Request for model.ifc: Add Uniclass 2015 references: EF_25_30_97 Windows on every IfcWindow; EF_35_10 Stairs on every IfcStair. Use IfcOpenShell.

First a look at what the model holds.

```python
import ifcopenshell

model = ifcopenshell.open("model.ifc")
print(model.schema)
print("classifications:", [c.Name for c in model.by_type("IfcClassification")])
for ifc_class in ("IfcDoor", "IfcRoof", "IfcStair", "IfcWall", "IfcWindow"):
    print(ifc_class, len(model.by_type(ifc_class)))
```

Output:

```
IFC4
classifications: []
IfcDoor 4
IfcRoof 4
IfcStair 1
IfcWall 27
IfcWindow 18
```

```python
import ifcopenshell
import ifcopenshell.api.classification

model = ifcopenshell.open("model.ifc")

system = ifcopenshell.api.classification.add_classification(model, classification="Uniclass 2015")

codes = {
    "IfcWindow": ("EF_25_30_97", "Windows"),
    "IfcStair": ("EF_35_10", "Stairs"),
}
for ifc_class, (code, name) in codes.items():
    products = model.by_type(ifc_class)
    ifcopenshell.api.classification.add_reference(
        model, products=products, classification=system, identification=code, name=name
    )
    print(code, len(products))

model.write("model_edited.ifc")
```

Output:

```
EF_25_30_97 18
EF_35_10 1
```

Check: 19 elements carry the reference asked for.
